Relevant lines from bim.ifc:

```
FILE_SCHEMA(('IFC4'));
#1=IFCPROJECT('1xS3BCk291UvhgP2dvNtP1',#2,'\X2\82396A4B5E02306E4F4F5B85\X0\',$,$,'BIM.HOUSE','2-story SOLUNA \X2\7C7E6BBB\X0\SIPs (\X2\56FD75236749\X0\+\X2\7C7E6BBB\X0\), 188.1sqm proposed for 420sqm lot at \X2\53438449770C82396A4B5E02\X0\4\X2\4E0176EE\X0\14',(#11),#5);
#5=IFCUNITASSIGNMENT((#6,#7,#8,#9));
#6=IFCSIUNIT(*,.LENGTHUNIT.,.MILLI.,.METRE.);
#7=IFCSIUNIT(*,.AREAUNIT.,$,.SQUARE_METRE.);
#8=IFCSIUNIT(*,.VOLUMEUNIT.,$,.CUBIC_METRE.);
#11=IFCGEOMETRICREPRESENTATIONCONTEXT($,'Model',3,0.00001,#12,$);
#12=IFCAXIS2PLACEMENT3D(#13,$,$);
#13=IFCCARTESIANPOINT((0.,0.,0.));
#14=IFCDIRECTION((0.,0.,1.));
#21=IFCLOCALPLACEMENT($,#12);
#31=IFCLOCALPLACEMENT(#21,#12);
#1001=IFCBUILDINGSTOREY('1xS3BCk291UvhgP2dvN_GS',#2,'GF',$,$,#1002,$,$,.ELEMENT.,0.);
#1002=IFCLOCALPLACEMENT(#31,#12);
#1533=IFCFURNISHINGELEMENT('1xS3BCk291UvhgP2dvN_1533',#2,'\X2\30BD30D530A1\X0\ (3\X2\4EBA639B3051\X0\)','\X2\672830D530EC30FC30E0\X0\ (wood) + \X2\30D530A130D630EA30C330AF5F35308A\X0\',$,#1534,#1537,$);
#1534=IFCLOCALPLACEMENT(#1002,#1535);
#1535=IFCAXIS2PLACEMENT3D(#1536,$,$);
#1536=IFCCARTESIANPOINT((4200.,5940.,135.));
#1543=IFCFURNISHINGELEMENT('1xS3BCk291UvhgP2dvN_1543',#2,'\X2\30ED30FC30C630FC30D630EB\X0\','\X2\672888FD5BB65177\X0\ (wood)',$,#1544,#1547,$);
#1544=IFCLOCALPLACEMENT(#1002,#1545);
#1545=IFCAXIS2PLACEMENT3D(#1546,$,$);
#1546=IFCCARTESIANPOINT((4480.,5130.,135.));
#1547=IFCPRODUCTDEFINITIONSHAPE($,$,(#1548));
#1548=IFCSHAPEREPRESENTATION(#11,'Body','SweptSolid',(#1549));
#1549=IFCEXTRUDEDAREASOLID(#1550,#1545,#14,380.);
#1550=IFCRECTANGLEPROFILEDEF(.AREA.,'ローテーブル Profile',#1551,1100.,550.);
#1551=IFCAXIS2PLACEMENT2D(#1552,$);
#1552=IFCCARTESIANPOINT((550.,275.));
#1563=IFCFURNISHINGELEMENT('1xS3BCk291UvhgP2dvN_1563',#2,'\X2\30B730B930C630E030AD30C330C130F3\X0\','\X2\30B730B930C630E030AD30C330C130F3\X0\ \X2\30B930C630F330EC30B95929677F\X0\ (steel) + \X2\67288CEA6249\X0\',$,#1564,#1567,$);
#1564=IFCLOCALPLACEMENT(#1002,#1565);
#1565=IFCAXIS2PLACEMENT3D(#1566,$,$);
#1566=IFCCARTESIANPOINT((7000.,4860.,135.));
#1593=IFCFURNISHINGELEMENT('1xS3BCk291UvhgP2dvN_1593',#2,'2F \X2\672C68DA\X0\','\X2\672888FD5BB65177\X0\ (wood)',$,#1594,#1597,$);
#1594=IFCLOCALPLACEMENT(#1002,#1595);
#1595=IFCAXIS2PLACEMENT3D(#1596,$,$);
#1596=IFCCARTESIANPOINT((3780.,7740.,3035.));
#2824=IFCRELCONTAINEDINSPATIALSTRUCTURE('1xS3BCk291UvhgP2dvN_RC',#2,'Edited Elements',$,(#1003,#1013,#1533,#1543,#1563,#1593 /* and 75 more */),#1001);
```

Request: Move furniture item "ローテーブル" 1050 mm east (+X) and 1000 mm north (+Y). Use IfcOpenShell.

```python
import ifcopenshell
import ifcopenshell.api.geometry
import ifcopenshell.util.placement
import ifcopenshell.util.unit

model = ifcopenshell.open("bim.ifc")
unit_scale = ifcopenshell.util.unit.calculate_unit_scale(model)

item = model.by_guid("1xS3BCk291UvhgP2dvN_1543")
matrix = ifcopenshell.util.placement.get_local_placement(item.ObjectPlacement)
matrix[0, 3] += 1.05 / unit_scale
matrix[1, 3] += 1 / unit_scale
ifcopenshell.api.geometry.edit_object_placement(model, product=item, matrix=matrix, is_si=False)

print(ifcopenshell.util.placement.get_local_placement(item.ObjectPlacement).round(3) + 0.0)

model.write("bim_rev.ifc")
```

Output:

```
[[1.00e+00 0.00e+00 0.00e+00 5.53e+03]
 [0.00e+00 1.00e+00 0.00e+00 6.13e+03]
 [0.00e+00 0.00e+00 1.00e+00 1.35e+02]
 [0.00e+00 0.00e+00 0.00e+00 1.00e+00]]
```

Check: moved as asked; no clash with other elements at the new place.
